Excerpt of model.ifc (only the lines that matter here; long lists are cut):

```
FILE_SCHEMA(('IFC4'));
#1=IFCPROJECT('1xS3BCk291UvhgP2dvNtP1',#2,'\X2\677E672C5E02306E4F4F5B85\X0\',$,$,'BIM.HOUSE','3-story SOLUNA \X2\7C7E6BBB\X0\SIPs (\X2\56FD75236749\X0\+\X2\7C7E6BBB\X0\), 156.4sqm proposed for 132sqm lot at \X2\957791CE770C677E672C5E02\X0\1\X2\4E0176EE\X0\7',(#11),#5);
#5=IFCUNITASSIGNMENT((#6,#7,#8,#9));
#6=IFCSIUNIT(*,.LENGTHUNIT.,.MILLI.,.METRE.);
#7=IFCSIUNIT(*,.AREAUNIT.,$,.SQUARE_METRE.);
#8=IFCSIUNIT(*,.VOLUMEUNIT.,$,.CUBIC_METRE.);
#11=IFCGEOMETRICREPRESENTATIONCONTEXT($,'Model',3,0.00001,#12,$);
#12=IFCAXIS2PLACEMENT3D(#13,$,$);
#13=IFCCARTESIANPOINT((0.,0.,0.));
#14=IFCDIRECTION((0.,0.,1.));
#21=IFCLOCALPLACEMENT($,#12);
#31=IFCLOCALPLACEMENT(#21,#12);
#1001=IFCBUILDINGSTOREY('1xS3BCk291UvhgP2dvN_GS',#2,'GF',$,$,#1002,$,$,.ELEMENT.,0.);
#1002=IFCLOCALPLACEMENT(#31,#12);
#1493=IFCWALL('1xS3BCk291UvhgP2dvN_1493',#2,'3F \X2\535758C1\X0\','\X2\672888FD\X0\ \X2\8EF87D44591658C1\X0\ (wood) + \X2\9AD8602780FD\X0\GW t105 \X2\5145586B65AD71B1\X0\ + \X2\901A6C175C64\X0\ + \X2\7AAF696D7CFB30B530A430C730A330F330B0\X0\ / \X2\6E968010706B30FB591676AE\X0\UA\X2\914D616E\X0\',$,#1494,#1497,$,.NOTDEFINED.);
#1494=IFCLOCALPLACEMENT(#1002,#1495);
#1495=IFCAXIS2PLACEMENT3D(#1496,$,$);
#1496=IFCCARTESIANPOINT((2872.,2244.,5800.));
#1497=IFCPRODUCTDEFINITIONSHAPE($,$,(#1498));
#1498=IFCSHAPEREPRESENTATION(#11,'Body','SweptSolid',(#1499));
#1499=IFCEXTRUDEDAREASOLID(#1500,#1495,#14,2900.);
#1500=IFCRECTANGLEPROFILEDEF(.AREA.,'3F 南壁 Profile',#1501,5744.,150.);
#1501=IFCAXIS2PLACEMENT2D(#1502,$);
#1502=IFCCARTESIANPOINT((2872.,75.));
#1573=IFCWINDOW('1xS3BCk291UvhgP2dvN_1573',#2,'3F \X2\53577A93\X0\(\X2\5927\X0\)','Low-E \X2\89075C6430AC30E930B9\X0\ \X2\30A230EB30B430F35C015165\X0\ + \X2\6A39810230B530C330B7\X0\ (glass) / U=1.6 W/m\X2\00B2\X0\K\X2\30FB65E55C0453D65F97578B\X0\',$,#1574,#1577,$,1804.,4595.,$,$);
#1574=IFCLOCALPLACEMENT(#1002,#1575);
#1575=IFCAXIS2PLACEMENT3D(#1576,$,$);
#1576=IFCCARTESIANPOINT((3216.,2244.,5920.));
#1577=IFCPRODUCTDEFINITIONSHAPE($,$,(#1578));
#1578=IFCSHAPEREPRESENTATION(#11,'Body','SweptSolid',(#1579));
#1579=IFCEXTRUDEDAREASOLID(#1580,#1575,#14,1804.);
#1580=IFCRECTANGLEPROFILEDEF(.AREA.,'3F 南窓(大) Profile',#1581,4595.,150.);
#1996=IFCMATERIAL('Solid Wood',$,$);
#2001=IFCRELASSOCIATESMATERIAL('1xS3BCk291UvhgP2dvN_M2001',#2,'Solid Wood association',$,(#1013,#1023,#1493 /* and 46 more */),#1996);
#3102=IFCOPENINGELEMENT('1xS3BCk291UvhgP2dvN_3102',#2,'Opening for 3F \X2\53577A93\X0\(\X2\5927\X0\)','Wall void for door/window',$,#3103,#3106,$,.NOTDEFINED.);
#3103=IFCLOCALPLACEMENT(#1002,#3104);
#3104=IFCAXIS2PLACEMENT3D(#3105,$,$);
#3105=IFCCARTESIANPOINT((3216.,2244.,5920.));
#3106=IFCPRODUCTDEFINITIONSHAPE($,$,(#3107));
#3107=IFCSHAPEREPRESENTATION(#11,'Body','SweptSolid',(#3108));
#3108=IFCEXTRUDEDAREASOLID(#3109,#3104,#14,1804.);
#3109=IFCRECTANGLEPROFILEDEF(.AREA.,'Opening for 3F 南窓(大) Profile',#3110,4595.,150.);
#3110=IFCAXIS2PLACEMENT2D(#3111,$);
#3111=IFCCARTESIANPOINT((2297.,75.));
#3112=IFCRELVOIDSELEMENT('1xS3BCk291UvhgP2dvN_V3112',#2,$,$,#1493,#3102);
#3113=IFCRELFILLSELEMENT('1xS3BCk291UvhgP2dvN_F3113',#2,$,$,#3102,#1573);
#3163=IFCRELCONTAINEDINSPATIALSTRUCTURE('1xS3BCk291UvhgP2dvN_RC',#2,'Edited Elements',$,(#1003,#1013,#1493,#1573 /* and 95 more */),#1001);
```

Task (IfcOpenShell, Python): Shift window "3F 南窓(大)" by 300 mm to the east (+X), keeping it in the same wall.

```python
import ifcopenshell
import ifcopenshell.api.geometry
import ifcopenshell.util.placement
import ifcopenshell.util.unit

model = ifcopenshell.open("model.ifc")
unit_scale = ifcopenshell.util.unit.calculate_unit_scale(model)

window = model.by_id(1573)
opening = window.FillsVoids[0].RelatingOpeningElement
wall = opening.VoidsElements[0].RelatingBuildingElement

wall_matrix = ifcopenshell.util.placement.get_local_placement(wall.ObjectPlacement)
shift = wall_matrix[:3, 0] * 0.3 / unit_scale
before = ifcopenshell.util.placement.get_local_placement(window.ObjectPlacement)[:3, 3].copy()

# The window is not placed relative to its opening, so move both.
for product in (opening, window):
    matrix = ifcopenshell.util.placement.get_local_placement(product.ObjectPlacement)
    matrix[:3, 3] += shift
    ifcopenshell.api.geometry.edit_object_placement(model, product=product, matrix=matrix, is_si=False)

after = ifcopenshell.util.placement.get_local_placement(window.ObjectPlacement)[:3, 3]
print("window moved by", (after - before).round(3) + 0.0)

model.write("model_edited.ifc")
```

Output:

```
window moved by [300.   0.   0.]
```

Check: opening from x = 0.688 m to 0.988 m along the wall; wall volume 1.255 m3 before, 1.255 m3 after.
